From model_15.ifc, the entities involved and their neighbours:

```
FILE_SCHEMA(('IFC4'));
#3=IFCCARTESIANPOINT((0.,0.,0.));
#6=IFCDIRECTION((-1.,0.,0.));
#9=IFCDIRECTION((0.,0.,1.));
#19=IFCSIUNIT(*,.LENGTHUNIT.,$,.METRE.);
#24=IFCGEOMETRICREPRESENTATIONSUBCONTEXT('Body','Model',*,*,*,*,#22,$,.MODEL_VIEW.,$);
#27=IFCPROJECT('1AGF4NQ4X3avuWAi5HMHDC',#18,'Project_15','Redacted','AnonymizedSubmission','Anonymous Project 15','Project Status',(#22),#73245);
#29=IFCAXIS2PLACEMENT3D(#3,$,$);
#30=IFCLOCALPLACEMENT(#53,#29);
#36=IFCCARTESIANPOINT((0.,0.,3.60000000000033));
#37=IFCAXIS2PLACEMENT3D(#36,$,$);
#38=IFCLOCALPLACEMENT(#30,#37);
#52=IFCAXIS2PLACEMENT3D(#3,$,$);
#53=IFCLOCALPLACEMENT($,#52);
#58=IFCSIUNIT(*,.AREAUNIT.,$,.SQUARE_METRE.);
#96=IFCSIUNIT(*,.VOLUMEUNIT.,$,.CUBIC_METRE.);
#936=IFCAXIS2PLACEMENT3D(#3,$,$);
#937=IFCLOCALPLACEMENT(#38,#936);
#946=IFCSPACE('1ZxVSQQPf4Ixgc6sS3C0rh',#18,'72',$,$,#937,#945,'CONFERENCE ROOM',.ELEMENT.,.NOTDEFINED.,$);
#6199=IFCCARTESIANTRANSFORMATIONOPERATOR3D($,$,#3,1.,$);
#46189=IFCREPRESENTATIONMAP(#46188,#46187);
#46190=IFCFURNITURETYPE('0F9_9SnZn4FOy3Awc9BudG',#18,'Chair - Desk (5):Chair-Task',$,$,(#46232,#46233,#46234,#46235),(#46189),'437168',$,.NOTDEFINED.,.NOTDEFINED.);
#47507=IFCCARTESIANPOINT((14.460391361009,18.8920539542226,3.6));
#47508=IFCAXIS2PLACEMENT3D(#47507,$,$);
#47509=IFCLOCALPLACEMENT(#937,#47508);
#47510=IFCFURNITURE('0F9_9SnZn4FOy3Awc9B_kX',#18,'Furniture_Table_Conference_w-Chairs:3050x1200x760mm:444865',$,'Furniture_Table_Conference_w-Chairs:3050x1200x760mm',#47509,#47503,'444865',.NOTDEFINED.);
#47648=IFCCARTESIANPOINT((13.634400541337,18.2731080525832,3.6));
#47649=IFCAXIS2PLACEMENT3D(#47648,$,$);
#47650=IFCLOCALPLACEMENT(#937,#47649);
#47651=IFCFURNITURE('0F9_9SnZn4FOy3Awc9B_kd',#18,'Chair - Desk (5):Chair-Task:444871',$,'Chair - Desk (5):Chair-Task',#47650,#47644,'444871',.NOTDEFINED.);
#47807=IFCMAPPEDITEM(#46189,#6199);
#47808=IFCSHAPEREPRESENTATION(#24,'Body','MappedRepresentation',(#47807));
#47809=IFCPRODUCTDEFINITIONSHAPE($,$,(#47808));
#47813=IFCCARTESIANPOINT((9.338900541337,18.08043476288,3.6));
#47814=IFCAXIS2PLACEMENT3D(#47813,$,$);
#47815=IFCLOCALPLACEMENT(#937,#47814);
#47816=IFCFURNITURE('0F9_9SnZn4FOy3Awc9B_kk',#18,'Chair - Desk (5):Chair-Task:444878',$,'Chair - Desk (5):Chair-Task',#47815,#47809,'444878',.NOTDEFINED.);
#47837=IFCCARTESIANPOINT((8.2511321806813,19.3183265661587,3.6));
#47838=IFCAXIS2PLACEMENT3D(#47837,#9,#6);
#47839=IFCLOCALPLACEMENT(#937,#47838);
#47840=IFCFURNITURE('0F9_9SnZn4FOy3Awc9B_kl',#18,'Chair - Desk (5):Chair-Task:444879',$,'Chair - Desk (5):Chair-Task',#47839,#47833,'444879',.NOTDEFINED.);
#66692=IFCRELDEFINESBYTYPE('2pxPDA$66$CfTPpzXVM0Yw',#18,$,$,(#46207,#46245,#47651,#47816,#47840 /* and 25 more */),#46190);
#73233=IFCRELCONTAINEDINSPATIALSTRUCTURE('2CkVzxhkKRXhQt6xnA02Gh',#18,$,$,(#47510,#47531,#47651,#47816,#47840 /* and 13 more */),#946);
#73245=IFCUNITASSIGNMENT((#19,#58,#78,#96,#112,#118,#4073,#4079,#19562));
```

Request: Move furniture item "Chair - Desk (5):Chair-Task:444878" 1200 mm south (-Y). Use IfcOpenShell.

```python
import ifcopenshell
import ifcopenshell.api.geometry
import ifcopenshell.util.placement

model = ifcopenshell.open("model_15.ifc")

item = model.by_id(47816)
matrix = ifcopenshell.util.placement.get_local_placement(item.ObjectPlacement)
matrix[1, 3] -= 1.2
ifcopenshell.api.geometry.edit_object_placement(model, product=item, matrix=matrix, is_si=False)

print(ifcopenshell.util.placement.get_local_placement(item.ObjectPlacement).round(3) + 0.0)

model.write("model_15-out.ifc")
```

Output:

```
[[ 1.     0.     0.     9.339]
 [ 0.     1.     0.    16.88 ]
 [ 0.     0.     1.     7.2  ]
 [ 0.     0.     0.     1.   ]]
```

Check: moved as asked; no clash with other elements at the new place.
